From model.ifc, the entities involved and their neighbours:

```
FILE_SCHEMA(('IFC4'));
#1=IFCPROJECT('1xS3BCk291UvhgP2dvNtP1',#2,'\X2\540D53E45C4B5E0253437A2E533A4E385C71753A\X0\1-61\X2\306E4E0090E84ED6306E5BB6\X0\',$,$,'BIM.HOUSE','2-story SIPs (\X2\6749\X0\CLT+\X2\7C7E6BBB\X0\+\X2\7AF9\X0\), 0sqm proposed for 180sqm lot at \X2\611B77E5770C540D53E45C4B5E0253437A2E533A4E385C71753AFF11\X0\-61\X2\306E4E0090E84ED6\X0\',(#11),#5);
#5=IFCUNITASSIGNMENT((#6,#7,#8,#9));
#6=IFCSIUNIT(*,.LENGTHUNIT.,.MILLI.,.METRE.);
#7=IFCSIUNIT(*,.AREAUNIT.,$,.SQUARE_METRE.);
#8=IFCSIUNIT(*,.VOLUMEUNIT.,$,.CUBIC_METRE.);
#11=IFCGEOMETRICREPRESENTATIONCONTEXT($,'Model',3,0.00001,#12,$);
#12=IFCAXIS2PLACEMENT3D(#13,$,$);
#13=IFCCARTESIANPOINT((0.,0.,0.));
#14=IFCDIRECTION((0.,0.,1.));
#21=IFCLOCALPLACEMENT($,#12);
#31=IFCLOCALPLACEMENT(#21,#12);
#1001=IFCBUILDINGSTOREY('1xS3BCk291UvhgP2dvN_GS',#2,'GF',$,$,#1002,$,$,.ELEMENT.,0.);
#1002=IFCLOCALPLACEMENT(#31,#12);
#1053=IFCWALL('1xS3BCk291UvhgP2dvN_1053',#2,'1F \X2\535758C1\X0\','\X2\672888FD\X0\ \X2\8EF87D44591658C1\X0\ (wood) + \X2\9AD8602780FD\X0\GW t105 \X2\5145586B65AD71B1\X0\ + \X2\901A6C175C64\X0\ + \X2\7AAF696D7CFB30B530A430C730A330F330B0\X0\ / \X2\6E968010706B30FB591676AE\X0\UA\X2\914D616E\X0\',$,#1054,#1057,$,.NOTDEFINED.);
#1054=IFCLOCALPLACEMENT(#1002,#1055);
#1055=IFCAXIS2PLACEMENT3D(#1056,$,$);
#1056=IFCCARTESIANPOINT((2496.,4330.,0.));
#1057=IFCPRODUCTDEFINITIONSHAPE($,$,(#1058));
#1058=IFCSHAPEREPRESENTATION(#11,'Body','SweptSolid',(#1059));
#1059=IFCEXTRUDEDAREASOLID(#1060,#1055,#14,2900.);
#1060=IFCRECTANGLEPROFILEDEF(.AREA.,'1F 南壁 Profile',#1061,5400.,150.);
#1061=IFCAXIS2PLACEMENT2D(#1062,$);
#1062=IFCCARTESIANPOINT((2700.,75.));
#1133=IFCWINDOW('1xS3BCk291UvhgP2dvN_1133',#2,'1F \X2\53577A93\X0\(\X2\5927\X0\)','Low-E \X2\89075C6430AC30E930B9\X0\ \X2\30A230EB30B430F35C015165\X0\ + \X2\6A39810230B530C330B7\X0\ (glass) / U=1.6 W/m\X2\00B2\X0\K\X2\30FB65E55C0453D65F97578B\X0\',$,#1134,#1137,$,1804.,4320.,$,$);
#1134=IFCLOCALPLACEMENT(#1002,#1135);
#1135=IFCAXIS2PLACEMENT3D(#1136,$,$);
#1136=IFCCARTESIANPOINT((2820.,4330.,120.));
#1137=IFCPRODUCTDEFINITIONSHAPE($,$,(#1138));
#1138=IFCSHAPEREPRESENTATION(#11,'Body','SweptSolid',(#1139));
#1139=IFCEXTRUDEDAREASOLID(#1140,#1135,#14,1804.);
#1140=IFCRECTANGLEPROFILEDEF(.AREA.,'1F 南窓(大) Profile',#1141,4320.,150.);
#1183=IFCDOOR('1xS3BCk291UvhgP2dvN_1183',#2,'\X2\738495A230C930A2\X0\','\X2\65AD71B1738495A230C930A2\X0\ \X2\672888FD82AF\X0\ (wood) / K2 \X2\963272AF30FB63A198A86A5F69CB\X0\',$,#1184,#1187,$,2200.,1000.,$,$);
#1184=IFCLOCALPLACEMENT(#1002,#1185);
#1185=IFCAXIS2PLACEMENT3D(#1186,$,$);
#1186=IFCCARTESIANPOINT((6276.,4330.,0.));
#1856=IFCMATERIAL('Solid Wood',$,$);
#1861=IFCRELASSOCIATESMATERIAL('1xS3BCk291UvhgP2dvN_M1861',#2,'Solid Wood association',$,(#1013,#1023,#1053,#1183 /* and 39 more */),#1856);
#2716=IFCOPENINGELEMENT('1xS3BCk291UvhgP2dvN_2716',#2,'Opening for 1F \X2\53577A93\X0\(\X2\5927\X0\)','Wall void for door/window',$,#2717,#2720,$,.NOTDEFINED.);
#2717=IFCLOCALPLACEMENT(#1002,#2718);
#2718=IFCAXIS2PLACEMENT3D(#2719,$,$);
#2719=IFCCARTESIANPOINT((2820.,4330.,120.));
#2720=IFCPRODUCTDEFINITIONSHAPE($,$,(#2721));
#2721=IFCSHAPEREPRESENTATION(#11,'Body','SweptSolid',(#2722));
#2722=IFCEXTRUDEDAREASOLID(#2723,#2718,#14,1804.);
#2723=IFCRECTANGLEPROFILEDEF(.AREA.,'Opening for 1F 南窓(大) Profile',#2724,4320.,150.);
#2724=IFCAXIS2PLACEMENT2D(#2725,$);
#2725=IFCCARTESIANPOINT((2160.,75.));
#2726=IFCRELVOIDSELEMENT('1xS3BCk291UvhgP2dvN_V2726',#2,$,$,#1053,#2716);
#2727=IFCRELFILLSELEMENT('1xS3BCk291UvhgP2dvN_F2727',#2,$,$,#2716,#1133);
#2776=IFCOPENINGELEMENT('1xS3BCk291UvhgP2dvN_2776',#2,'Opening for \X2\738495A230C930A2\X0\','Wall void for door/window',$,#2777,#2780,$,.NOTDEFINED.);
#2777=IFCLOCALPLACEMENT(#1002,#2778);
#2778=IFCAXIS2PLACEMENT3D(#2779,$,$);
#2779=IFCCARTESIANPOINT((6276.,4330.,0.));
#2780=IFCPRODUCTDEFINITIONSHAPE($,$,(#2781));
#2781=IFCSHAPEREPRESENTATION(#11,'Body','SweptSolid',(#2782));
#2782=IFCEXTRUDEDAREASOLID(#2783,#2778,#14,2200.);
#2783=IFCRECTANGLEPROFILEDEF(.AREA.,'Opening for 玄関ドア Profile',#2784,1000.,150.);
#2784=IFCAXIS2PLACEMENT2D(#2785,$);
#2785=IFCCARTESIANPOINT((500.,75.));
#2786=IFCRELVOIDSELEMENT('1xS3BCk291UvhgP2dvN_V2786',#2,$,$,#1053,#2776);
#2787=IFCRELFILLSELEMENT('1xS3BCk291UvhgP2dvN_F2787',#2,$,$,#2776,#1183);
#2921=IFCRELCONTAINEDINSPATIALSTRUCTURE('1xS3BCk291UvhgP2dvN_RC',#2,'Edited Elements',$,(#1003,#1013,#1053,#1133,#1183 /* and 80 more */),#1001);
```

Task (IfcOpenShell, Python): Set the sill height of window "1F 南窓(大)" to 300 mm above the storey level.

```python
import numpy as np
import ifcopenshell
import ifcopenshell.api.geometry
import ifcopenshell.geom
import ifcopenshell.util.element
import ifcopenshell.util.placement
import ifcopenshell.util.shape
import ifcopenshell.util.unit

model = ifcopenshell.open("model.ifc")
unit_scale = ifcopenshell.util.unit.calculate_unit_scale(model)

window = model.by_id(1133)
opening = window.FillsVoids[0].RelatingOpeningElement
storey = ifcopenshell.util.element.get_container(window, ifc_class="IfcBuildingStorey")
level = ifcopenshell.util.placement.get_local_placement(storey.ObjectPlacement)[2, 3]

# The opening's origin need not be at the sill, so measure its lowest point.
shape = ifcopenshell.geom.create_shape(ifcopenshell.geom.settings(), opening)
bottom = ifcopenshell.util.shape.get_shape_bottom_elevation(shape, shape.geometry) / unit_scale
dz = level + 0.3 / unit_scale - bottom

shift = np.array([0.0, 0.0, dz])
# The window is not placed relative to its opening, so move both.
for product in (opening, window):
    matrix = ifcopenshell.util.placement.get_local_placement(product.ObjectPlacement)
    matrix[:3, 3] += shift
    ifcopenshell.api.geometry.edit_object_placement(model, product=product, matrix=matrix, is_si=False)

print(f"moved by {dz * unit_scale:+.3f} m")

model.write("model_rev.ifc")
```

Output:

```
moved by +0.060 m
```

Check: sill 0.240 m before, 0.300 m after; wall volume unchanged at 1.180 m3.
